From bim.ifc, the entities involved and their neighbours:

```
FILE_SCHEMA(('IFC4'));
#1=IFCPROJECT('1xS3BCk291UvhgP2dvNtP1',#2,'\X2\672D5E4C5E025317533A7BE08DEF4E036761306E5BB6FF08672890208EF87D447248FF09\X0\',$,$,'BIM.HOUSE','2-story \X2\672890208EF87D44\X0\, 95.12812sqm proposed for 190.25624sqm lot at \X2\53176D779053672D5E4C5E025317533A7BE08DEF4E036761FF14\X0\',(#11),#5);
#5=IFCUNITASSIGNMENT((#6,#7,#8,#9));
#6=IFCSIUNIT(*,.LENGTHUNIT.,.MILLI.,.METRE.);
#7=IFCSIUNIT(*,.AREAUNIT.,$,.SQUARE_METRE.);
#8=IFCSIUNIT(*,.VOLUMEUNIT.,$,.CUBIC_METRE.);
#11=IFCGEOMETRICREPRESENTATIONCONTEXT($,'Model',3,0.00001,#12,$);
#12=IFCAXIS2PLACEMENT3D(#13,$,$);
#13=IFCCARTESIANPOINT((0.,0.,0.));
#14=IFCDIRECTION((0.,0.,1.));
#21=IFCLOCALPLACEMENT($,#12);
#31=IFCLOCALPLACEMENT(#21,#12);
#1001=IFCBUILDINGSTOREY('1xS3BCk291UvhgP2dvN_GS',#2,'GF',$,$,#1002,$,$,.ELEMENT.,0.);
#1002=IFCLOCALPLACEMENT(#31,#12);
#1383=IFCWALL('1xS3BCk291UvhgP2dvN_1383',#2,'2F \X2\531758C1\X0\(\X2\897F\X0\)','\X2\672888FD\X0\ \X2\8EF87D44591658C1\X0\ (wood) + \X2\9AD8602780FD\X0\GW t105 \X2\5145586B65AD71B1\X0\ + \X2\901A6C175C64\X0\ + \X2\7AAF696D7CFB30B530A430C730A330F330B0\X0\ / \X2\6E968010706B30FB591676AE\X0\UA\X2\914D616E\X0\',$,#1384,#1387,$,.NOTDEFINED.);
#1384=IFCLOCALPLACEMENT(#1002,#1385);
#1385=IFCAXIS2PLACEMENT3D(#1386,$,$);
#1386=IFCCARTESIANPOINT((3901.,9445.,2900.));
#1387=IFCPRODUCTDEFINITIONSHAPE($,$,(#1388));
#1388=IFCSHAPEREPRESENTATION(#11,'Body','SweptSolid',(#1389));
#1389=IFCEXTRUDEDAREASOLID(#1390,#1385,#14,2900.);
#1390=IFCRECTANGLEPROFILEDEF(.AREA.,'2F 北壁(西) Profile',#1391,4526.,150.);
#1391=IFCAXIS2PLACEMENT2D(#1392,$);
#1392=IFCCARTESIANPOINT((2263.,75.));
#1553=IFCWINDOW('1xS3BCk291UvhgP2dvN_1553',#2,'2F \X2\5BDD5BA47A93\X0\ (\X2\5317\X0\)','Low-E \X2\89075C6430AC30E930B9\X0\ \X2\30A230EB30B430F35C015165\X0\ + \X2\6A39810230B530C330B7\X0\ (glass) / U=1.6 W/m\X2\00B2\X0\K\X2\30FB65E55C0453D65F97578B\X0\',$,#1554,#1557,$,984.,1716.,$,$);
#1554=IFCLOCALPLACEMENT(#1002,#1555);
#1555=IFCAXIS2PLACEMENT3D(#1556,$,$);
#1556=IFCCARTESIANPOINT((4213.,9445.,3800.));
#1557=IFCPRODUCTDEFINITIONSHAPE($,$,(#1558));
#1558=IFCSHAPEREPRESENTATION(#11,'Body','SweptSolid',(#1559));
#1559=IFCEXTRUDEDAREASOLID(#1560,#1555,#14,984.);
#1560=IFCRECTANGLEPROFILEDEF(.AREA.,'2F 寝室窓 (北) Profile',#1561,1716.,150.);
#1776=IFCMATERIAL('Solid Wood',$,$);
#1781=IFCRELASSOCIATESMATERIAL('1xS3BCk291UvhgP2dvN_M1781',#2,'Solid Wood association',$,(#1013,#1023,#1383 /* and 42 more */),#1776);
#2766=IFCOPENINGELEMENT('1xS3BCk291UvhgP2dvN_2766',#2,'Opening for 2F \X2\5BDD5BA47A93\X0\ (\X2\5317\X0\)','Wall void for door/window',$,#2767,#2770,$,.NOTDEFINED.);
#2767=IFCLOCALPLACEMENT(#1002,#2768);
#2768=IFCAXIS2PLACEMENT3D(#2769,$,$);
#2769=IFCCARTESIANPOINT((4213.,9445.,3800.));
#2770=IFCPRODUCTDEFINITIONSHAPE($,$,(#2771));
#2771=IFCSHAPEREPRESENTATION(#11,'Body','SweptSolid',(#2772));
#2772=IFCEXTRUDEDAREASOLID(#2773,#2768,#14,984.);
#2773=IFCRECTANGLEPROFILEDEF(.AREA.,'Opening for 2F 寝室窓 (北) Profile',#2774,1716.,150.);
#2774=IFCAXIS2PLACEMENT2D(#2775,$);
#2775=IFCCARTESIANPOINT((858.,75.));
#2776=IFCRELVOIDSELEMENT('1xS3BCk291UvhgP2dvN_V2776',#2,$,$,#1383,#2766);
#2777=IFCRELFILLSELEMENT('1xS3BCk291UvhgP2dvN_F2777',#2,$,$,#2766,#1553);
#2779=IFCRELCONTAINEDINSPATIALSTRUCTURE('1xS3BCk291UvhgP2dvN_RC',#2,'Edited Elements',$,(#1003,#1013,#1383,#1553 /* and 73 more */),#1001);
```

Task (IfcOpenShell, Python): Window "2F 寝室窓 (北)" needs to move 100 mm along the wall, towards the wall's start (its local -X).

```python
import ifcopenshell
import ifcopenshell.api.geometry
import ifcopenshell.util.placement
import ifcopenshell.util.unit

model = ifcopenshell.open("bim.ifc")
unit_scale = ifcopenshell.util.unit.calculate_unit_scale(model)

window = model.by_guid("1xS3BCk291UvhgP2dvN_1553")
opening = window.FillsVoids[0].RelatingOpeningElement
wall = opening.VoidsElements[0].RelatingBuildingElement

wall_matrix = ifcopenshell.util.placement.get_local_placement(wall.ObjectPlacement)
shift = wall_matrix[:3, 0] * -0.1 / unit_scale
before = ifcopenshell.util.placement.get_local_placement(window.ObjectPlacement)[:3, 3].copy()

# The window is not placed relative to its opening, so move both.
for product in (opening, window):
    matrix = ifcopenshell.util.placement.get_local_placement(product.ObjectPlacement)
    matrix[:3, 3] += shift
    ifcopenshell.api.geometry.edit_object_placement(model, product=product, matrix=matrix, is_si=False)

after = ifcopenshell.util.placement.get_local_placement(window.ObjectPlacement)[:3, 3]
print("window moved by", (after - before).round(3) + 0.0)

model.write("bim_rev.ifc")
```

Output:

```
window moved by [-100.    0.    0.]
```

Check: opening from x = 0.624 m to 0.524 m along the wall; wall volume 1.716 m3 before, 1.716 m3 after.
